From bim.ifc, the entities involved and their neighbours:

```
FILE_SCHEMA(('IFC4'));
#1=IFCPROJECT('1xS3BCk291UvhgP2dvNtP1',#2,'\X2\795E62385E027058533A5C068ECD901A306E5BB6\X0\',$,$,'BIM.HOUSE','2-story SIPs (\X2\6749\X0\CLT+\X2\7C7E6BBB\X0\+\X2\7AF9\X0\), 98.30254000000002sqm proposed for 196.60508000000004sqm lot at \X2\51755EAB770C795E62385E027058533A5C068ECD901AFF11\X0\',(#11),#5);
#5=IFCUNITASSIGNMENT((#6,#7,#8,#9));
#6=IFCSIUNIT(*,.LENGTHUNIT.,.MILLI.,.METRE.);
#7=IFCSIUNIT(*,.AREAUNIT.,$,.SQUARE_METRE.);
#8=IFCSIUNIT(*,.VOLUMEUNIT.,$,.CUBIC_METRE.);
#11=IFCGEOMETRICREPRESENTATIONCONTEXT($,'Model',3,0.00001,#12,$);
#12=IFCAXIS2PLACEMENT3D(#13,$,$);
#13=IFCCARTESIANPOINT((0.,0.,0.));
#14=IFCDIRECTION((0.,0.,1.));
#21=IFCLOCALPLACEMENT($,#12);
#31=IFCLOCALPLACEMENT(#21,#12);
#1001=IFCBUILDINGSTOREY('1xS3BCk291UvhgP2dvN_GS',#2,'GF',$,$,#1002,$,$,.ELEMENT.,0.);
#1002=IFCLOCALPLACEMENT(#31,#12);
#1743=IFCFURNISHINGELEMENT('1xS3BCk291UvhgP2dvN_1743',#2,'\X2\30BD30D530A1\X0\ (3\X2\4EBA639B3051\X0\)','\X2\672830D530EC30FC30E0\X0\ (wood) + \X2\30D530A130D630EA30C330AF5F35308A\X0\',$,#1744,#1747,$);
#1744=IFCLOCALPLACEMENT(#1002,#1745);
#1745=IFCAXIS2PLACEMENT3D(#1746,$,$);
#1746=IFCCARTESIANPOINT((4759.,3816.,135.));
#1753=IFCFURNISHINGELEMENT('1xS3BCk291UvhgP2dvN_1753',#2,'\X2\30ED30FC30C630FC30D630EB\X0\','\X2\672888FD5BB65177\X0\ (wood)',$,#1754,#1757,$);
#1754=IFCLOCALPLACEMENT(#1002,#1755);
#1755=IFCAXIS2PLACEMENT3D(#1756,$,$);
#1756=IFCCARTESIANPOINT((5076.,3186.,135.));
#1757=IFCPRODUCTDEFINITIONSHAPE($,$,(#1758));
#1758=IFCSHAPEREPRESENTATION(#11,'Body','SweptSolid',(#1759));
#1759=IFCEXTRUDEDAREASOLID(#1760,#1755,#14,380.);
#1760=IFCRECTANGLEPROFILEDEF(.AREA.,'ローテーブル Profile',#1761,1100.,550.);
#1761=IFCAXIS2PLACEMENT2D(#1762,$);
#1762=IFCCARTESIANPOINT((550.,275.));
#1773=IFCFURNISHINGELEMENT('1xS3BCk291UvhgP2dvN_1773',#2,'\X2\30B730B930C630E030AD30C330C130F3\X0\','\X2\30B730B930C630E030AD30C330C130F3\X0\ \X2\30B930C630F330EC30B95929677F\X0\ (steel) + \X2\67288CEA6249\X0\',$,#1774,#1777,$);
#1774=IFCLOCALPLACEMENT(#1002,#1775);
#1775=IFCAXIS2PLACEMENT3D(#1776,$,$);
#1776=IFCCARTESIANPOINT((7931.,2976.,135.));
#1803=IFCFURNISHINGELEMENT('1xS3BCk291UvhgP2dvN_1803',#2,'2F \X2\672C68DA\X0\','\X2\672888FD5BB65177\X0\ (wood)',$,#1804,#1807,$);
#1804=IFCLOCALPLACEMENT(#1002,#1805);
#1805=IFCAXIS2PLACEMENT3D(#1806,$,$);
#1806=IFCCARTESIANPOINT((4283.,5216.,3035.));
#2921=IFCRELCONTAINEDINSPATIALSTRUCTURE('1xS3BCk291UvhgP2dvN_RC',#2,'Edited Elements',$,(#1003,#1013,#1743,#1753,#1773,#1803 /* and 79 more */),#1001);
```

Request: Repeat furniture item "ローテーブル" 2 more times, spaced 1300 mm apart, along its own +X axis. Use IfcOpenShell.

```python
import ifcopenshell
import ifcopenshell.api.geometry
import ifcopenshell.api.root
import ifcopenshell.util.element
import ifcopenshell.util.placement
import ifcopenshell.util.unit

model = ifcopenshell.open("bim.ifc")
unit_scale = ifcopenshell.util.unit.calculate_unit_scale(model)


def reuse_history(source, copy):
    """copy_class also copies each property set's owner history, people and application; keep the originals."""
    for rel in copy.IsDefinedBy:
        if rel.is_a("IfcRelDefinesByProperties") and (history := rel.RelatingPropertyDefinition.OwnerHistory):
            rel.RelatingPropertyDefinition.OwnerHistory = source.OwnerHistory
            ifcopenshell.util.element.remove_deep2(model, history)


source = model.by_id(1753)
base = ifcopenshell.util.placement.get_local_placement(source.ObjectPlacement)
step = base[:3, 0] * 1.3 / unit_scale

for i in range(1, 3):
    copy = ifcopenshell.api.root.copy_class(model, product=source)
    copy.Representation = ifcopenshell.util.element.copy_deep(
        model, source.Representation, exclude=["IfcGeometricRepresentationContext", "IfcRepresentationMap"]
    )
    reuse_history(source, copy)
    matrix = base.copy()
    matrix[:3, 3] += i * step
    print("added at", matrix[:3, 3].round(3) + 0.0)
    ifcopenshell.api.geometry.edit_object_placement(model, product=copy, matrix=matrix, is_si=False)

model.write("bim_v2.ifc")
```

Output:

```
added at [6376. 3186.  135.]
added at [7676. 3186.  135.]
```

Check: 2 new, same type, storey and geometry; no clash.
